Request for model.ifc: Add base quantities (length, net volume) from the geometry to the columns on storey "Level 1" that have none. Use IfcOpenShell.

First a look at what the model holds.

```python
import ifcopenshell
import ifcopenshell.util.element
import ifcopenshell.util.unit

model = ifcopenshell.open("model.ifc")
print(model.schema)
for unit_type in ("LENGTHUNIT", "AREAUNIT", "VOLUMEUNIT"):
    print(unit_type, ifcopenshell.util.unit.calculate_unit_scale(model, unit_type))
storey = next(s for s in model.by_type("IfcBuildingStorey") if s.Name == "Level 1")
columns = [e for e in ifcopenshell.util.element.get_decomposition(storey) if e.is_a("IfcColumn")]
for e in sorted(columns, key=lambda e: e.id()):
    print(e.id(), e.is_a(), e.Name, list(ifcopenshell.util.element.get_psets(e, qtos_only=True)), sep=" | ")
```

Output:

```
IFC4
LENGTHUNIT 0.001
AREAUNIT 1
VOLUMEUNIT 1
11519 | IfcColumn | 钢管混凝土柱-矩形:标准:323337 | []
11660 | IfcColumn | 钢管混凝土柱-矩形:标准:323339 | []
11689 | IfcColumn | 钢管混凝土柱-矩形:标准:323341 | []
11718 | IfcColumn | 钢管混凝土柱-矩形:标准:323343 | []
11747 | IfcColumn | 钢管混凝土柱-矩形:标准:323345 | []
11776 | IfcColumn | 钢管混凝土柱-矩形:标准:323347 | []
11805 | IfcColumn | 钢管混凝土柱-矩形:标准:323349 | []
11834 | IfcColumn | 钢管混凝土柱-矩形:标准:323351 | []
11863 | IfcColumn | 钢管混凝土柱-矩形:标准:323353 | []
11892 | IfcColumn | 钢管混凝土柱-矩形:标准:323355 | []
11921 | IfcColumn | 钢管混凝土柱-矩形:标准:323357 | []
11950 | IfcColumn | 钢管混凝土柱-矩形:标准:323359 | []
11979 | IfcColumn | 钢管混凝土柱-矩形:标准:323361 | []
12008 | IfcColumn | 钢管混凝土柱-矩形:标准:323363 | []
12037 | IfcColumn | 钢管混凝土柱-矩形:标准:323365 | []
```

```python
import ifcopenshell
import ifcopenshell.api.pset
import ifcopenshell.geom
import ifcopenshell.util.element
import ifcopenshell.util.shape
import ifcopenshell.util.unit

model = ifcopenshell.open("model.ifc")
unit_scale = ifcopenshell.util.unit.calculate_unit_scale(model)
volume_scale = ifcopenshell.util.unit.calculate_unit_scale(model, "VOLUMEUNIT")
settings = ifcopenshell.geom.settings()

storey = next(s for s in model.by_type("IfcBuildingStorey") if s.Name == "Level 1")
columns = [e for e in ifcopenshell.util.element.get_decomposition(storey) if e.is_a("IfcColumn")]

for e in sorted(columns, key=lambda e: e.id()):
    if ifcopenshell.util.element.get_psets(e, qtos_only=True, should_inherit=False):
        continue
    # Geometry comes back in metres, in the element's own axes.
    shape = ifcopenshell.geom.create_shape(settings, e)
    values = {
        "Length": ifcopenshell.util.shape.get_z(shape.geometry) / unit_scale,
        "NetVolume": ifcopenshell.util.shape.get_volume(shape.geometry) / volume_scale,
    }
    qto = ifcopenshell.api.pset.add_qto(model, product=e, name="Qto_ColumnBaseQuantities")
    ifcopenshell.api.pset.edit_qto(model, qto=qto, properties=values)
    print(e.id(), {k: round(v, 3) for k, v in values.items()})

model.write("model-out.ifc")
```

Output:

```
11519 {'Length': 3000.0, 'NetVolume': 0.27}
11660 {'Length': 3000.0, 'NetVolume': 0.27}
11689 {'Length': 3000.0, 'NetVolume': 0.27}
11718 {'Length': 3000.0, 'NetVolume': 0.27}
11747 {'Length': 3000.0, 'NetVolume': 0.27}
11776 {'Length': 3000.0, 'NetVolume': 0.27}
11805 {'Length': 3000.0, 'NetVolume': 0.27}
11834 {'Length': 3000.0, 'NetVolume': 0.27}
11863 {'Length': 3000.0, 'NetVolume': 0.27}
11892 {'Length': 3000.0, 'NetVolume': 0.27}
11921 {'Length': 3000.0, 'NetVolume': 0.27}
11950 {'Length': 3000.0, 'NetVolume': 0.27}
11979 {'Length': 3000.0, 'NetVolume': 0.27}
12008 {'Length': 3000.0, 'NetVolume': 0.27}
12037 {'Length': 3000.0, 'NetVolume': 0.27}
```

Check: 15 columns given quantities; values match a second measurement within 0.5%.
